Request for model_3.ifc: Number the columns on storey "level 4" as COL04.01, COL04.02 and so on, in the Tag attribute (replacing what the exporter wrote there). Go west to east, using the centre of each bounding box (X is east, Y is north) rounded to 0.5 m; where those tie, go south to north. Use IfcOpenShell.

First a look at what the model holds.

```python
import ifcopenshell
import ifcopenshell.util.element
import ifcopenshell.util.placement

model = ifcopenshell.open("model_3.ifc")
print(model.schema)
storey = next(s for s in model.by_type("IfcBuildingStorey") if s.Name == "level 4")
columns = [e for e in ifcopenshell.util.element.get_decomposition(storey) if e.is_a("IfcColumn")]
for e in sorted(columns, key=lambda e: e.id()):
    origin = ifcopenshell.util.placement.get_local_placement(e.ObjectPlacement)[:3, 3]
    print(e.id(), e.Tag, e.Name, origin.round(2) + 0.0, sep=" | ")
```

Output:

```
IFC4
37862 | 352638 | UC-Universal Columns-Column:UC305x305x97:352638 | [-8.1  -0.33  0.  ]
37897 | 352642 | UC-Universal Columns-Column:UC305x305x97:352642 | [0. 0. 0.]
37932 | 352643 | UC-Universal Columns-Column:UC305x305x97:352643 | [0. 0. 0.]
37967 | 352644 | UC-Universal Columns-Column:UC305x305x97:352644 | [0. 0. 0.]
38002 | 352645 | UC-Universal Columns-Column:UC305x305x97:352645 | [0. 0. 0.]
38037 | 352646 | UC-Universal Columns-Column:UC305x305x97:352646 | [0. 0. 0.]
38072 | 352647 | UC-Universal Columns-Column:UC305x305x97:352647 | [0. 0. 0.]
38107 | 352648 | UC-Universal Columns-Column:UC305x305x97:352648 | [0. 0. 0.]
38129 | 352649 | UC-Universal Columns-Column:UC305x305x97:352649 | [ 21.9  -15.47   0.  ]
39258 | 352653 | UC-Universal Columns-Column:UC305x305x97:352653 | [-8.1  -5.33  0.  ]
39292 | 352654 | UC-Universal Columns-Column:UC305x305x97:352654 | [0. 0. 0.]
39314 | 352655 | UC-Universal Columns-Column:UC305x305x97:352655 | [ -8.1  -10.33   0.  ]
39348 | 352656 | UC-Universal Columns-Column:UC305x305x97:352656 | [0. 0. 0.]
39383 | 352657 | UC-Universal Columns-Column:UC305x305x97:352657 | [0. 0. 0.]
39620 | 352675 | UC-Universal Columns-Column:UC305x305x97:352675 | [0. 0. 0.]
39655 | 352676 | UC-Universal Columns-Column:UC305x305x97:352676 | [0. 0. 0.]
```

```python
import ifcopenshell
import ifcopenshell.geom
import ifcopenshell.util.element
import ifcopenshell.util.shape

model = ifcopenshell.open("model_3.ifc")
settings = ifcopenshell.geom.settings()
settings.set("use-world-coords", True)


def centre(element):
    shape = ifcopenshell.geom.create_shape(settings, element)
    return ifcopenshell.util.shape.get_bbox_centroid(shape.geometry)


storey = next(s for s in model.by_type("IfcBuildingStorey") if s.Name == "level 4")
columns = [e for e in ifcopenshell.util.element.get_decomposition(storey) if e.is_a("IfcColumn")]

# Insertion points can sit at a corner or the storey origin, so sort by the geometry (in metres).
centres = {e: centre(e) for e in columns}
columns.sort(key=lambda e: (round(centres[e][0] / 0.5), centres[e][1]))

for i, e in enumerate(columns, start=1):
    number = f"COL04.{i:02d}"
    e.Tag = number
    print(e.id(), number)

model.write("model_3_rev.ifc")
```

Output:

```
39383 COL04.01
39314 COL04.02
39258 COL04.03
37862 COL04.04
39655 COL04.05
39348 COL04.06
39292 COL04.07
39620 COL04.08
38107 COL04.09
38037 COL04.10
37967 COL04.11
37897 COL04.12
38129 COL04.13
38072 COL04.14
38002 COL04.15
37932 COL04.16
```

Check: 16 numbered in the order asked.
